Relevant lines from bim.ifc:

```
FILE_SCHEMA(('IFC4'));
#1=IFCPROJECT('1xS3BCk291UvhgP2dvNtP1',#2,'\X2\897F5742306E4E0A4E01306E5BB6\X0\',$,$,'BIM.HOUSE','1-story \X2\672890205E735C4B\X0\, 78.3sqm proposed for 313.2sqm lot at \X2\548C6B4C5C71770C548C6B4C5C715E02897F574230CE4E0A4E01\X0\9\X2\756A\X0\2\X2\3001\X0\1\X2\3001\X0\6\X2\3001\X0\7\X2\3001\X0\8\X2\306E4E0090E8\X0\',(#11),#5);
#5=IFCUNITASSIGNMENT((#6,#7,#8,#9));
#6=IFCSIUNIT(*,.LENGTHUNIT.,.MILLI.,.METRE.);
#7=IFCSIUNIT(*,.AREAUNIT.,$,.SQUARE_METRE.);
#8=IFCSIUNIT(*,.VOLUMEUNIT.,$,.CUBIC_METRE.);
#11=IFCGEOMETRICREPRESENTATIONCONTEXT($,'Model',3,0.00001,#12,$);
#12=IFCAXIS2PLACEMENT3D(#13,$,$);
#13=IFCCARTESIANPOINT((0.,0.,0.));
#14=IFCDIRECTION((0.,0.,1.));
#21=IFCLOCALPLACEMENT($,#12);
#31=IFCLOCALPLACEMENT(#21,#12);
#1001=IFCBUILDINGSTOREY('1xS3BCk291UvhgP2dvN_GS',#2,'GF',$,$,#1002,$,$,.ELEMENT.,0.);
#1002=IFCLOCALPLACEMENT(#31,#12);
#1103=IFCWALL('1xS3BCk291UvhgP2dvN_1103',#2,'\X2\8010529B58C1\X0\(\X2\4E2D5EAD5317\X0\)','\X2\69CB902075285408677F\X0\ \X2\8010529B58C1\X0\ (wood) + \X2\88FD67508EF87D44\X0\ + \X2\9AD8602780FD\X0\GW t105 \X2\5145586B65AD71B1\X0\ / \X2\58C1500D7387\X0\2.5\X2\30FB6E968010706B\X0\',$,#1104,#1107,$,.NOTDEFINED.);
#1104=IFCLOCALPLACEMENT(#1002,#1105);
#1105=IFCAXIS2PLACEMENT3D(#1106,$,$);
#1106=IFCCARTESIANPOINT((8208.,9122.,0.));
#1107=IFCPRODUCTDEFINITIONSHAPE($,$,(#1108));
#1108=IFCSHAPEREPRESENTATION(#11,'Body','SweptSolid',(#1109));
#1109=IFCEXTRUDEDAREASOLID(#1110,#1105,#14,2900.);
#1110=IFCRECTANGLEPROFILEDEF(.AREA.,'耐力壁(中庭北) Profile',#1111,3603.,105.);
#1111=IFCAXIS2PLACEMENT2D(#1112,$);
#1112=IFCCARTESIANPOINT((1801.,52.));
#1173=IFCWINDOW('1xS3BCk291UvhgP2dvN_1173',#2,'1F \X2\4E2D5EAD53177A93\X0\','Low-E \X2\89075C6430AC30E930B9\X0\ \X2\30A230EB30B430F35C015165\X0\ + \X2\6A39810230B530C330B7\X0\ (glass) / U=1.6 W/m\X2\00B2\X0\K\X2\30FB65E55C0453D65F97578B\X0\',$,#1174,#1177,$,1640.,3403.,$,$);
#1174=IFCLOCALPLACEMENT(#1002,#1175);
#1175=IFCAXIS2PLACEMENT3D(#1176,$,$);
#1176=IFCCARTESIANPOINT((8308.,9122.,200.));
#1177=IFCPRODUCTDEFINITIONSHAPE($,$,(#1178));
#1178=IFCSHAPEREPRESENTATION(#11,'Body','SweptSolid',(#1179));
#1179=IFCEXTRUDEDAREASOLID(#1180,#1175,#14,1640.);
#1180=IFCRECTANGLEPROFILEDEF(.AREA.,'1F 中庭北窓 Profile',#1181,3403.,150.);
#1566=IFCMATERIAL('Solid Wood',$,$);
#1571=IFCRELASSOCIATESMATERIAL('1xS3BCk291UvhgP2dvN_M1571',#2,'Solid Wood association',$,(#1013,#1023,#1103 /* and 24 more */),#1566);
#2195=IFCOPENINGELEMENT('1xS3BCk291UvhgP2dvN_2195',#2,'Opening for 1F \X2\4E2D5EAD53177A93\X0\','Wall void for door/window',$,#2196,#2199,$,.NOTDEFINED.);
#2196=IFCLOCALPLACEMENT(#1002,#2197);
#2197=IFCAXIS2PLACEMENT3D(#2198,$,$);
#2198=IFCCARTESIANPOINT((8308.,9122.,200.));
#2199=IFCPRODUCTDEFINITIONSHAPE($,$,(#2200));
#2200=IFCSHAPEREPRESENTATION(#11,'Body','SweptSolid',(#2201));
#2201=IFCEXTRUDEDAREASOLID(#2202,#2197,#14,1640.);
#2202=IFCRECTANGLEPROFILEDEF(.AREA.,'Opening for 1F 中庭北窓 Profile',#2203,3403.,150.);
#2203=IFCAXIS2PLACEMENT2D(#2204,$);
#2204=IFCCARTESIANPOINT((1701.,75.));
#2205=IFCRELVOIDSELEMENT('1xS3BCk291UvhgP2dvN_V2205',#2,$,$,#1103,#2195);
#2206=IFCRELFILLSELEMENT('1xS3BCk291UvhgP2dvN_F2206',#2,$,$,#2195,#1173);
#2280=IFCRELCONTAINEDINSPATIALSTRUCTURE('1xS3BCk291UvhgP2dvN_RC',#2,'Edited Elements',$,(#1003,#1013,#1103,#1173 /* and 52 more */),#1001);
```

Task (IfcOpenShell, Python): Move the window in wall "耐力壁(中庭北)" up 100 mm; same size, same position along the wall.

```python
import numpy as np
import ifcopenshell
import ifcopenshell.api.geometry
import ifcopenshell.util.placement
import ifcopenshell.util.unit

model = ifcopenshell.open("bim.ifc")
unit_scale = ifcopenshell.util.unit.calculate_unit_scale(model)

window = model.by_guid("1xS3BCk291UvhgP2dvN_1173")
opening = window.FillsVoids[0].RelatingOpeningElement
dz = 0.1 / unit_scale

shift = np.array([0.0, 0.0, dz])
# The window is not placed relative to its opening, so move both.
for product in (opening, window):
    matrix = ifcopenshell.util.placement.get_local_placement(product.ObjectPlacement)
    matrix[:3, 3] += shift
    ifcopenshell.api.geometry.edit_object_placement(model, product=product, matrix=matrix, is_si=False)

print(f"moved by {dz * unit_scale:+.3f} m")

model.write("bim_updated.ifc")
```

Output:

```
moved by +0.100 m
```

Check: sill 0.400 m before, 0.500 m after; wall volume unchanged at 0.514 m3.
